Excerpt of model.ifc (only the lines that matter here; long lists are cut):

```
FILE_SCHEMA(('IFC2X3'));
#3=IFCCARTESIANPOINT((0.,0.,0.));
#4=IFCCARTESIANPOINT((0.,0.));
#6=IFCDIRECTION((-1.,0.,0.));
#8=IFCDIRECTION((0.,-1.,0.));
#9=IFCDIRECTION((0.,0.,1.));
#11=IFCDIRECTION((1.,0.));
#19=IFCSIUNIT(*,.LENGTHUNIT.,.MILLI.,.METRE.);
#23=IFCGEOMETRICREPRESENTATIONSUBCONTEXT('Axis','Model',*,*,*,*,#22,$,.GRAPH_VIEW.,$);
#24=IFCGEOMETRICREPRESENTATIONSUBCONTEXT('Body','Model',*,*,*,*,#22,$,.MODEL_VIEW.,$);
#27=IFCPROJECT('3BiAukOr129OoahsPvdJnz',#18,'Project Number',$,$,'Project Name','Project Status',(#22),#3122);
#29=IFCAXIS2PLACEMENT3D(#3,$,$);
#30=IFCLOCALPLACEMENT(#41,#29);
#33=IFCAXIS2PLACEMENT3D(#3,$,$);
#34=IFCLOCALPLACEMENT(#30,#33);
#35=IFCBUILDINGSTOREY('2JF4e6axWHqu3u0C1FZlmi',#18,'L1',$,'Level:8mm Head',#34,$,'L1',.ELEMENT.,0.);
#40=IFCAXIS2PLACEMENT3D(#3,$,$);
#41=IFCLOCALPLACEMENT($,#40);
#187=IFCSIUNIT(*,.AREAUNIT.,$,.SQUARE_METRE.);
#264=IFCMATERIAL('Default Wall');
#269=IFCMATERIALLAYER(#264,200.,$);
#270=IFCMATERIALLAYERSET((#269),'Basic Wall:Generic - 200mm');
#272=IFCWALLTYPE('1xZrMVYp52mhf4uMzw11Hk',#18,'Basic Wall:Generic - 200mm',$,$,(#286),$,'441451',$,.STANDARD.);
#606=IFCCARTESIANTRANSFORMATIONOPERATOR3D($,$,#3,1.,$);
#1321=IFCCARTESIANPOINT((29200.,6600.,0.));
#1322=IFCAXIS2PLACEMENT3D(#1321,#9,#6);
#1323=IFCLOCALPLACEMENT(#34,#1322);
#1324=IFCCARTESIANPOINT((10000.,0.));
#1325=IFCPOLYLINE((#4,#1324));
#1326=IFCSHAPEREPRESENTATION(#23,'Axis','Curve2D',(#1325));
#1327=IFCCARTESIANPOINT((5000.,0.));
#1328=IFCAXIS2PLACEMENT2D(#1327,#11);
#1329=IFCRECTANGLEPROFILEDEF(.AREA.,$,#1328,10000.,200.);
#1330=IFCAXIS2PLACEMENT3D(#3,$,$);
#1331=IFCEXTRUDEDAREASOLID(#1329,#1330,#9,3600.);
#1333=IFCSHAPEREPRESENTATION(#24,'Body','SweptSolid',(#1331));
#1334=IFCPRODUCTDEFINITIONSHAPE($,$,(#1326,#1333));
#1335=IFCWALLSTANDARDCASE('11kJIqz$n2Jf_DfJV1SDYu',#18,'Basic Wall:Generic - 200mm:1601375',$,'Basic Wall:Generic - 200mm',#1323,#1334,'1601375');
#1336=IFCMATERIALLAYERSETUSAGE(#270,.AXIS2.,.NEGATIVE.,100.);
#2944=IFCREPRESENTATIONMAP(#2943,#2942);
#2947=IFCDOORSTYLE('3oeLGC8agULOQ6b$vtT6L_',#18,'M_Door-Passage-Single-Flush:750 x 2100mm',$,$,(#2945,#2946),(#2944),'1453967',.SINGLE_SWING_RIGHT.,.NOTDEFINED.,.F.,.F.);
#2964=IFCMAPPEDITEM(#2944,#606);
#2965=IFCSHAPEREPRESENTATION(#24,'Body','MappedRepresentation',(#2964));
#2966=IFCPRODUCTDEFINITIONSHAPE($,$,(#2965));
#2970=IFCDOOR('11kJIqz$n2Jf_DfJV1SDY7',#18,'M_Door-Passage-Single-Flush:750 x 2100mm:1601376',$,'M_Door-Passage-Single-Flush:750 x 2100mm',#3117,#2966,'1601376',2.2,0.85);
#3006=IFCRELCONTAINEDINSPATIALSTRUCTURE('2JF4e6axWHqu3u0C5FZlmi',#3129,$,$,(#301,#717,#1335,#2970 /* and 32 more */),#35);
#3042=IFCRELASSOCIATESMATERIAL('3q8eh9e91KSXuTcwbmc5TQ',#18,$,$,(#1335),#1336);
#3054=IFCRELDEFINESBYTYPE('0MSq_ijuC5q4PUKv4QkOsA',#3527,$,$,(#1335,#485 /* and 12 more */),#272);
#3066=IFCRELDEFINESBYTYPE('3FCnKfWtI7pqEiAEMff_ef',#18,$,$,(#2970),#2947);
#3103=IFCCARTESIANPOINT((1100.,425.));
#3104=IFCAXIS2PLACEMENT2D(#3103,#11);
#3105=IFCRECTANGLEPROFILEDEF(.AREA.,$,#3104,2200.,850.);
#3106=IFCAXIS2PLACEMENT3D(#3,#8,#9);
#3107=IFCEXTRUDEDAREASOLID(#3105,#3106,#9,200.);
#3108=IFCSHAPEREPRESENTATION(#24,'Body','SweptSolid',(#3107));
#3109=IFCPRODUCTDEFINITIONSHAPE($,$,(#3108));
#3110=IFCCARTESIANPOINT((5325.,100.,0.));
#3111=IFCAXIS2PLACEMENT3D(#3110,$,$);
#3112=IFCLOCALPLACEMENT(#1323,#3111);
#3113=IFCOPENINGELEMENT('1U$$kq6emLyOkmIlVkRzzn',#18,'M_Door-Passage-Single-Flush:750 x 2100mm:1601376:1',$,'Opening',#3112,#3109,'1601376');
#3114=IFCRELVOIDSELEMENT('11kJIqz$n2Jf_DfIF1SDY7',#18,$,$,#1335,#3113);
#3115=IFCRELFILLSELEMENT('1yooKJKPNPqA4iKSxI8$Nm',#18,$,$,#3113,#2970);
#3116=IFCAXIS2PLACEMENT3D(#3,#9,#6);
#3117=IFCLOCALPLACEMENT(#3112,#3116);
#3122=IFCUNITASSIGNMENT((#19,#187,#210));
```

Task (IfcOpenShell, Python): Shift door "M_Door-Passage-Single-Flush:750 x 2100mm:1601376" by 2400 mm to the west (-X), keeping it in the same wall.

```python
import ifcopenshell
import ifcopenshell.api.geometry
import ifcopenshell.util.placement
import ifcopenshell.util.unit

model = ifcopenshell.open("model.ifc")
unit_scale = ifcopenshell.util.unit.calculate_unit_scale(model)

door = model.by_id(2970)
opening = door.FillsVoids[0].RelatingOpeningElement
wall = opening.VoidsElements[0].RelatingBuildingElement

wall_matrix = ifcopenshell.util.placement.get_local_placement(wall.ObjectPlacement)
shift = wall_matrix[:3, 0] * 2.4 / unit_scale
before = ifcopenshell.util.placement.get_local_placement(door.ObjectPlacement)[:3, 3].copy()

# The door is placed relative to its opening, so it follows when the opening moves.
matrix = ifcopenshell.util.placement.get_local_placement(opening.ObjectPlacement)
matrix[:3, 3] += shift
ifcopenshell.api.geometry.edit_object_placement(
    model, product=opening, matrix=matrix, is_si=False, should_transform_children=True
)

after = ifcopenshell.util.placement.get_local_placement(door.ObjectPlacement)[:3, 3]
print("door moved by", (after - before).round(3) + 0.0)

model.write("model_updated.ifc")
```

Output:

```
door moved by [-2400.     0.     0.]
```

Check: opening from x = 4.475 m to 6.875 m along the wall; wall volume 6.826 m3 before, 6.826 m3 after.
